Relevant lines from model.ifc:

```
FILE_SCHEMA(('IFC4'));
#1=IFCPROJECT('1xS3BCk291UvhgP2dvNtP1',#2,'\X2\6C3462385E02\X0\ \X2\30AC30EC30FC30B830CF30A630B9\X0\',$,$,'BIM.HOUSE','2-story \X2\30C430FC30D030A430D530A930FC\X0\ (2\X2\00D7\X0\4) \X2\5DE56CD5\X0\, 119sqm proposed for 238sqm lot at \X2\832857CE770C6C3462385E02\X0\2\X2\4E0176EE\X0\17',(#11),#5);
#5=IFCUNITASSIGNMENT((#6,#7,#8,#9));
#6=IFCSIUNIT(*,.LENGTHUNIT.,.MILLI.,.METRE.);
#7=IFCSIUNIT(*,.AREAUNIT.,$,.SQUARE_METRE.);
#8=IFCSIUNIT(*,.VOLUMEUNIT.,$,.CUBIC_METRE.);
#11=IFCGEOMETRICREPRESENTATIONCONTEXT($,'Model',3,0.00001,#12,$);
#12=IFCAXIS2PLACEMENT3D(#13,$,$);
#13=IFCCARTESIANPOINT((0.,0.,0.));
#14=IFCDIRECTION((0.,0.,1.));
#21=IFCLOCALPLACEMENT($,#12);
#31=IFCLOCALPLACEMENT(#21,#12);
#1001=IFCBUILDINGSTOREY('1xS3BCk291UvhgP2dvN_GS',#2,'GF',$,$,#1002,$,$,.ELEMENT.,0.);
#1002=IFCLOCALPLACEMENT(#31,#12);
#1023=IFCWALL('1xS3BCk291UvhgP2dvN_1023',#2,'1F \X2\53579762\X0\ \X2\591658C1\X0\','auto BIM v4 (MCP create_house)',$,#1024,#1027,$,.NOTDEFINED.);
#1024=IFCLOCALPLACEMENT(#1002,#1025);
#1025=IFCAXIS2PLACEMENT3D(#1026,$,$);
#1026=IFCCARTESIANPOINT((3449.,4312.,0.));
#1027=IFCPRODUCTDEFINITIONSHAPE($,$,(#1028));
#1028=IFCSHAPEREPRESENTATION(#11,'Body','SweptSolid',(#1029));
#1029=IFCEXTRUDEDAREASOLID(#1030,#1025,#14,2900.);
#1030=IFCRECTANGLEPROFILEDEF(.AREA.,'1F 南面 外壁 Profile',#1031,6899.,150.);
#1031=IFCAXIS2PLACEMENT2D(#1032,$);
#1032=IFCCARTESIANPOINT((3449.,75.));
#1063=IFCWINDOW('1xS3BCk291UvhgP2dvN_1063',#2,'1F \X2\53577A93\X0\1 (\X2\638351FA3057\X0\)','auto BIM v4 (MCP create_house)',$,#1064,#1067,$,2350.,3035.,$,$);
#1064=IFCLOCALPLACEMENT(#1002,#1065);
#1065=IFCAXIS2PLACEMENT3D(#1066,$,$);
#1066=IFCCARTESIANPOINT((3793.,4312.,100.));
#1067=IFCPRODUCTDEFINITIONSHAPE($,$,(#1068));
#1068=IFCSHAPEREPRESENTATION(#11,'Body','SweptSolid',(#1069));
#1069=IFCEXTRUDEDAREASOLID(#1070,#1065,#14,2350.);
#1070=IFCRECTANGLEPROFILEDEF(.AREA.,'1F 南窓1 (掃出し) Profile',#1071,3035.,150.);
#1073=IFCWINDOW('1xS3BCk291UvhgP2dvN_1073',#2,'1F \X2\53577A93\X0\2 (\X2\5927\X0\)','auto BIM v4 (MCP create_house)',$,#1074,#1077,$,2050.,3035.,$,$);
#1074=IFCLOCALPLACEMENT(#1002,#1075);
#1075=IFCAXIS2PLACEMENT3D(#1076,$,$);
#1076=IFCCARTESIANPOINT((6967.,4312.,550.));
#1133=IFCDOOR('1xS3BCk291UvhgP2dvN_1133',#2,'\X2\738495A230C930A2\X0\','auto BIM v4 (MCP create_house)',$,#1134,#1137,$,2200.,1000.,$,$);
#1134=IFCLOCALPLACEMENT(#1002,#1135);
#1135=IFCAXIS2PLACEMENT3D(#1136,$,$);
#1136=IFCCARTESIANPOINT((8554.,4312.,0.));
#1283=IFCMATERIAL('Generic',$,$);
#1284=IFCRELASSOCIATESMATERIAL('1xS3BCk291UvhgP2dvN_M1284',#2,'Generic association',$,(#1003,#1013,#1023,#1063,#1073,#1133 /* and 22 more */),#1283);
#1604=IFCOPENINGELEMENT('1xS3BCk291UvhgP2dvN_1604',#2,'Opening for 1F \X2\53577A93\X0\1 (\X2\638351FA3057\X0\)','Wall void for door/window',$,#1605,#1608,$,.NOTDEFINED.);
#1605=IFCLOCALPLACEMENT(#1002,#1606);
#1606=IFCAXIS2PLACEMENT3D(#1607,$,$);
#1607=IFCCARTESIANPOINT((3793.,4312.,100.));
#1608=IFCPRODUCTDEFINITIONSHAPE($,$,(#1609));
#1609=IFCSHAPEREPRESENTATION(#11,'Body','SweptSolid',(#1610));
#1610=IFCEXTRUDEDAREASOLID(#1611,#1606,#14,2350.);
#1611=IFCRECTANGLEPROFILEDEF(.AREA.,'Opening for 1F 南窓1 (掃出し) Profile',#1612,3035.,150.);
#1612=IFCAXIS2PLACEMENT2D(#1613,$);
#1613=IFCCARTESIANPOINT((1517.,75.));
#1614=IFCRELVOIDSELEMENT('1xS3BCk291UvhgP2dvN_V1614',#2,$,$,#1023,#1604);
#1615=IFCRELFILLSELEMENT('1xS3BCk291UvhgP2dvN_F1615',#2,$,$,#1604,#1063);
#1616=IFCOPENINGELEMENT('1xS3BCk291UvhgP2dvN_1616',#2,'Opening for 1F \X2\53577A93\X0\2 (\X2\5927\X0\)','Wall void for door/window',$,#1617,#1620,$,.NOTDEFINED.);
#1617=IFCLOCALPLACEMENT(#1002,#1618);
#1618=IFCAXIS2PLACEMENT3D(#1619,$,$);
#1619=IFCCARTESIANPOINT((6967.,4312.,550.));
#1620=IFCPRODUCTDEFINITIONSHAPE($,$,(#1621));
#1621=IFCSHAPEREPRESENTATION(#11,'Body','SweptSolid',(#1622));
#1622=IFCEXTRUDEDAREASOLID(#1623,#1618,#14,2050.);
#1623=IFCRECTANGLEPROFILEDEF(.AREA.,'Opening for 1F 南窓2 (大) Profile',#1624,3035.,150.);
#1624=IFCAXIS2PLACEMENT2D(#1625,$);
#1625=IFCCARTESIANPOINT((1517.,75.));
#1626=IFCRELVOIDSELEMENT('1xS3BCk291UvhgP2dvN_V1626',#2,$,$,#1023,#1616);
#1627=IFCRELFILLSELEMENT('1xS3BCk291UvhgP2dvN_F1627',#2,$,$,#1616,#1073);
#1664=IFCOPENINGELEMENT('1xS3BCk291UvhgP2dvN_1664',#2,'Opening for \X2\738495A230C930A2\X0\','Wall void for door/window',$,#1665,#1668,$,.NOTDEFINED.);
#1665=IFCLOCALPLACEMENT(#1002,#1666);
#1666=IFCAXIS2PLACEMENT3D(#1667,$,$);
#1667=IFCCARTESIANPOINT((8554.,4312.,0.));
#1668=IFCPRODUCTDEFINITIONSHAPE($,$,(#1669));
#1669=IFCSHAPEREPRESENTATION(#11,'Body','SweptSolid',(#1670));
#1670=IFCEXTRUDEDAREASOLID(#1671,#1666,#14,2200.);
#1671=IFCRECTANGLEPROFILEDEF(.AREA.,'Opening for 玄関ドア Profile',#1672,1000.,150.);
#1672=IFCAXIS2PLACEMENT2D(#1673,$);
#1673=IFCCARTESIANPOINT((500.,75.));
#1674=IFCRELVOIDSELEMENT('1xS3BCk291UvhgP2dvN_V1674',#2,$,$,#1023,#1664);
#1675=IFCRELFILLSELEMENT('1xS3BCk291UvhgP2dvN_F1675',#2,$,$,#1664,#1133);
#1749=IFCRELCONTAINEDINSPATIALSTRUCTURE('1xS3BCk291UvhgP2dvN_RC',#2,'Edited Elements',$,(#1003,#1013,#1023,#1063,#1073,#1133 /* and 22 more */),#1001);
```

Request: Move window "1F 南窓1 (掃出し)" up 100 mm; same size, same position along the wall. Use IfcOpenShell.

```python
import numpy as np
import ifcopenshell
import ifcopenshell.api.geometry
import ifcopenshell.util.placement
import ifcopenshell.util.unit

model = ifcopenshell.open("model.ifc")
unit_scale = ifcopenshell.util.unit.calculate_unit_scale(model)

window = model.by_id(1063)
opening = window.FillsVoids[0].RelatingOpeningElement
dz = 0.1 / unit_scale

shift = np.array([0.0, 0.0, dz])
# The window is not placed relative to its opening, so move both.
for product in (opening, window):
    matrix = ifcopenshell.util.placement.get_local_placement(product.ObjectPlacement)
    matrix[:3, 3] += shift
    ifcopenshell.api.geometry.edit_object_placement(model, product=product, matrix=matrix, is_si=False)

print(f"moved by {dz * unit_scale:+.3f} m")

model.write("model_updated.ifc")
```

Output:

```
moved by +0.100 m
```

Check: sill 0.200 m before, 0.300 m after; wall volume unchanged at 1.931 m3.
